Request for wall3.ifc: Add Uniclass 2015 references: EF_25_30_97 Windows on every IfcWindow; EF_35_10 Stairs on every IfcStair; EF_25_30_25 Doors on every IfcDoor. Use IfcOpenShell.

First a look at what the model holds.

```python
import ifcopenshell

model = ifcopenshell.open("wall3.ifc")
print(model.schema)
print("classifications:", [c.Name for c in model.by_type("IfcClassification")])
for ifc_class in ("IfcDoor", "IfcRoof", "IfcStair", "IfcWall", "IfcWindow"):
    print(ifc_class, len(model.by_type(ifc_class)))
```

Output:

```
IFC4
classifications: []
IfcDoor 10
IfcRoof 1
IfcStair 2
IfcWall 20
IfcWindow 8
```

```python
import ifcopenshell
import ifcopenshell.api.classification

model = ifcopenshell.open("wall3.ifc")

system = ifcopenshell.api.classification.add_classification(model, classification="Uniclass 2015")

codes = {
    "IfcWindow": ("EF_25_30_97", "Windows"),
    "IfcStair": ("EF_35_10", "Stairs"),
    "IfcDoor": ("EF_25_30_25", "Doors"),
}
for ifc_class, (code, name) in codes.items():
    products = model.by_type(ifc_class)
    ifcopenshell.api.classification.add_reference(
        model, products=products, classification=system, identification=code, name=name
    )
    print(code, len(products))

model.write("wall3-out.ifc")
```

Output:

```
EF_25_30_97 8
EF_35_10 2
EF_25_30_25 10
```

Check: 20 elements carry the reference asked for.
